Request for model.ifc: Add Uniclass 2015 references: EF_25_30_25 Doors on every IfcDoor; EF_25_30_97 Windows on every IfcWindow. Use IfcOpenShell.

First a look at what the model holds.

```python
import ifcopenshell

model = ifcopenshell.open("model.ifc")
print(model.schema)
print("classifications:", [c.Name for c in model.by_type("IfcClassification")])
for ifc_class in ("IfcDoor", "IfcRoof", "IfcStair", "IfcWall", "IfcWindow"):
    print(ifc_class, len(model.by_type(ifc_class)))
```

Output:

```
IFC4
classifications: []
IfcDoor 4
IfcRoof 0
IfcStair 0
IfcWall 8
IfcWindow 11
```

```python
import ifcopenshell
import ifcopenshell.api.classification

model = ifcopenshell.open("model.ifc")

system = ifcopenshell.api.classification.add_classification(model, classification="Uniclass 2015")

codes = {
    "IfcDoor": ("EF_25_30_25", "Doors"),
    "IfcWindow": ("EF_25_30_97", "Windows"),
}
for ifc_class, (code, name) in codes.items():
    products = model.by_type(ifc_class)
    ifcopenshell.api.classification.add_reference(
        model, products=products, classification=system, identification=code, name=name
    )
    print(code, len(products))

model.write("model_rev.ifc")
```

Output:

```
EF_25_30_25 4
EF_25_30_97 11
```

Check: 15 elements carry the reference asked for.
